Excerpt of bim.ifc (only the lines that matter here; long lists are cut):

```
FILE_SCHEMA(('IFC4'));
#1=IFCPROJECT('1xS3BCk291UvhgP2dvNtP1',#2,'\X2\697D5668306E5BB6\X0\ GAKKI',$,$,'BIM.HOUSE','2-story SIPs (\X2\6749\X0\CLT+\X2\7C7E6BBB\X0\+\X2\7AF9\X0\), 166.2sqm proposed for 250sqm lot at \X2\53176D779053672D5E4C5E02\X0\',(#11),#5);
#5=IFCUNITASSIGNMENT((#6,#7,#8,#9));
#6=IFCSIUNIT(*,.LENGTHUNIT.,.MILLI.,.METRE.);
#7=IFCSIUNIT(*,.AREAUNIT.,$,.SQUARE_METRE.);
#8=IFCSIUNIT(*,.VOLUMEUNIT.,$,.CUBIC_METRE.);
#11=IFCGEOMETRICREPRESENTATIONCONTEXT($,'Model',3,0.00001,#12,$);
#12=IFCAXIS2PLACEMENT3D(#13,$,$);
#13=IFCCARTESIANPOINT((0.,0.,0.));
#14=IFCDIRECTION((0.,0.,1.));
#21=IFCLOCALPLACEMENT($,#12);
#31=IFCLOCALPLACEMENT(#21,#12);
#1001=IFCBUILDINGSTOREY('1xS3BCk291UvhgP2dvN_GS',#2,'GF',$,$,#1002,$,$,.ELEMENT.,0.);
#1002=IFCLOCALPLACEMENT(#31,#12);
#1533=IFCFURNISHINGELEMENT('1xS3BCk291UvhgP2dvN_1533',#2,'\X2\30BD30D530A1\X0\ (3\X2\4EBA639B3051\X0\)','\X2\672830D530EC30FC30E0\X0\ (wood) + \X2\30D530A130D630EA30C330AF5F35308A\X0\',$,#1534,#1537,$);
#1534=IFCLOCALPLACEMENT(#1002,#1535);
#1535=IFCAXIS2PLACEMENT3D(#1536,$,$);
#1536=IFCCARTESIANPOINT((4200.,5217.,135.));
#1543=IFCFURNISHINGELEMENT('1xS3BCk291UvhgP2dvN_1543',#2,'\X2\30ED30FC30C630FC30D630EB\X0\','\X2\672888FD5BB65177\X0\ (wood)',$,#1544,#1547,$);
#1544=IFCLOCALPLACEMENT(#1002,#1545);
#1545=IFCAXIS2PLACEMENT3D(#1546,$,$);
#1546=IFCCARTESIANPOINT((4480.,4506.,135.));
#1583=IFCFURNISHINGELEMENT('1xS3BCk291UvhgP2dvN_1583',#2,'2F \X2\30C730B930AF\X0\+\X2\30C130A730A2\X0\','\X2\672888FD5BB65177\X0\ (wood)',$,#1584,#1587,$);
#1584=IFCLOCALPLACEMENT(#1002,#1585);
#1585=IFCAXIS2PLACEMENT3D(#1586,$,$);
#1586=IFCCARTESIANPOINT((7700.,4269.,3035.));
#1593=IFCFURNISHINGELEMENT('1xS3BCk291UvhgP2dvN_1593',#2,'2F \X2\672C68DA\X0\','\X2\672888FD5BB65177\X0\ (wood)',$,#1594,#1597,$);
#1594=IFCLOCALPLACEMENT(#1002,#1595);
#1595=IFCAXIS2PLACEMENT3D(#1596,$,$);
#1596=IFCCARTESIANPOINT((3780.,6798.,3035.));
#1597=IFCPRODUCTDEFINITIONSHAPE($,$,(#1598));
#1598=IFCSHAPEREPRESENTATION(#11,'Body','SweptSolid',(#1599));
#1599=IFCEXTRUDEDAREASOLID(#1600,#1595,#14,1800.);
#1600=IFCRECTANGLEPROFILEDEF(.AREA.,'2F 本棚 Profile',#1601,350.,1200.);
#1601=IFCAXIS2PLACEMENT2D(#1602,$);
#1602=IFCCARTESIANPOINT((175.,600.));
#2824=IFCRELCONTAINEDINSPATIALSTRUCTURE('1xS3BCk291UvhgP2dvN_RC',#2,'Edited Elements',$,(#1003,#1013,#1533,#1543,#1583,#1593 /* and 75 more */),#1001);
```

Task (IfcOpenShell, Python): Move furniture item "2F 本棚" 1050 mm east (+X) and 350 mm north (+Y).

```python
import ifcopenshell
import ifcopenshell.api.geometry
import ifcopenshell.util.placement
import ifcopenshell.util.unit

model = ifcopenshell.open("bim.ifc")
unit_scale = ifcopenshell.util.unit.calculate_unit_scale(model)

item = model.by_guid("1xS3BCk291UvhgP2dvN_1593")
matrix = ifcopenshell.util.placement.get_local_placement(item.ObjectPlacement)
matrix[0, 3] += 1.05 / unit_scale
matrix[1, 3] += 0.35 / unit_scale
ifcopenshell.api.geometry.edit_object_placement(model, product=item, matrix=matrix, is_si=False)

print(ifcopenshell.util.placement.get_local_placement(item.ObjectPlacement).round(3) + 0.0)

model.write("bim_v2.ifc")
```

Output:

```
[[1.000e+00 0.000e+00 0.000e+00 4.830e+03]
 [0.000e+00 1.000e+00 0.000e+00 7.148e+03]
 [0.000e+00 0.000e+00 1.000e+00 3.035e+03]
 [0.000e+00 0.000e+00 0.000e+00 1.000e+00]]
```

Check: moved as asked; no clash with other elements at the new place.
